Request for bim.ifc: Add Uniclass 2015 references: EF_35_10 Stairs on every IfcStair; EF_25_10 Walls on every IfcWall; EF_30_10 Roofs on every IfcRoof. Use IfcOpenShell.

First a look at what the model holds.

```python
import ifcopenshell

model = ifcopenshell.open("bim.ifc")
print(model.schema)
print("classifications:", [c.Name for c in model.by_type("IfcClassification")])
for ifc_class in ("IfcDoor", "IfcRoof", "IfcStair", "IfcWall", "IfcWindow"):
    print(ifc_class, len(model.by_type(ifc_class)))
```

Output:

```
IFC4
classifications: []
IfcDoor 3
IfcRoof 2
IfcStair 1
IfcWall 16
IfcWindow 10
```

```python
import ifcopenshell
import ifcopenshell.api.classification

model = ifcopenshell.open("bim.ifc")

system = ifcopenshell.api.classification.add_classification(model, classification="Uniclass 2015")

codes = {
    "IfcStair": ("EF_35_10", "Stairs"),
    "IfcWall": ("EF_25_10", "Walls"),
    "IfcRoof": ("EF_30_10", "Roofs"),
}
for ifc_class, (code, name) in codes.items():
    products = model.by_type(ifc_class)
    ifcopenshell.api.classification.add_reference(
        model, products=products, classification=system, identification=code, name=name
    )
    print(code, len(products))

model.write("bim_v2.ifc")
```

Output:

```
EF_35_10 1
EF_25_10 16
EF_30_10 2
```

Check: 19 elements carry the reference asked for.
